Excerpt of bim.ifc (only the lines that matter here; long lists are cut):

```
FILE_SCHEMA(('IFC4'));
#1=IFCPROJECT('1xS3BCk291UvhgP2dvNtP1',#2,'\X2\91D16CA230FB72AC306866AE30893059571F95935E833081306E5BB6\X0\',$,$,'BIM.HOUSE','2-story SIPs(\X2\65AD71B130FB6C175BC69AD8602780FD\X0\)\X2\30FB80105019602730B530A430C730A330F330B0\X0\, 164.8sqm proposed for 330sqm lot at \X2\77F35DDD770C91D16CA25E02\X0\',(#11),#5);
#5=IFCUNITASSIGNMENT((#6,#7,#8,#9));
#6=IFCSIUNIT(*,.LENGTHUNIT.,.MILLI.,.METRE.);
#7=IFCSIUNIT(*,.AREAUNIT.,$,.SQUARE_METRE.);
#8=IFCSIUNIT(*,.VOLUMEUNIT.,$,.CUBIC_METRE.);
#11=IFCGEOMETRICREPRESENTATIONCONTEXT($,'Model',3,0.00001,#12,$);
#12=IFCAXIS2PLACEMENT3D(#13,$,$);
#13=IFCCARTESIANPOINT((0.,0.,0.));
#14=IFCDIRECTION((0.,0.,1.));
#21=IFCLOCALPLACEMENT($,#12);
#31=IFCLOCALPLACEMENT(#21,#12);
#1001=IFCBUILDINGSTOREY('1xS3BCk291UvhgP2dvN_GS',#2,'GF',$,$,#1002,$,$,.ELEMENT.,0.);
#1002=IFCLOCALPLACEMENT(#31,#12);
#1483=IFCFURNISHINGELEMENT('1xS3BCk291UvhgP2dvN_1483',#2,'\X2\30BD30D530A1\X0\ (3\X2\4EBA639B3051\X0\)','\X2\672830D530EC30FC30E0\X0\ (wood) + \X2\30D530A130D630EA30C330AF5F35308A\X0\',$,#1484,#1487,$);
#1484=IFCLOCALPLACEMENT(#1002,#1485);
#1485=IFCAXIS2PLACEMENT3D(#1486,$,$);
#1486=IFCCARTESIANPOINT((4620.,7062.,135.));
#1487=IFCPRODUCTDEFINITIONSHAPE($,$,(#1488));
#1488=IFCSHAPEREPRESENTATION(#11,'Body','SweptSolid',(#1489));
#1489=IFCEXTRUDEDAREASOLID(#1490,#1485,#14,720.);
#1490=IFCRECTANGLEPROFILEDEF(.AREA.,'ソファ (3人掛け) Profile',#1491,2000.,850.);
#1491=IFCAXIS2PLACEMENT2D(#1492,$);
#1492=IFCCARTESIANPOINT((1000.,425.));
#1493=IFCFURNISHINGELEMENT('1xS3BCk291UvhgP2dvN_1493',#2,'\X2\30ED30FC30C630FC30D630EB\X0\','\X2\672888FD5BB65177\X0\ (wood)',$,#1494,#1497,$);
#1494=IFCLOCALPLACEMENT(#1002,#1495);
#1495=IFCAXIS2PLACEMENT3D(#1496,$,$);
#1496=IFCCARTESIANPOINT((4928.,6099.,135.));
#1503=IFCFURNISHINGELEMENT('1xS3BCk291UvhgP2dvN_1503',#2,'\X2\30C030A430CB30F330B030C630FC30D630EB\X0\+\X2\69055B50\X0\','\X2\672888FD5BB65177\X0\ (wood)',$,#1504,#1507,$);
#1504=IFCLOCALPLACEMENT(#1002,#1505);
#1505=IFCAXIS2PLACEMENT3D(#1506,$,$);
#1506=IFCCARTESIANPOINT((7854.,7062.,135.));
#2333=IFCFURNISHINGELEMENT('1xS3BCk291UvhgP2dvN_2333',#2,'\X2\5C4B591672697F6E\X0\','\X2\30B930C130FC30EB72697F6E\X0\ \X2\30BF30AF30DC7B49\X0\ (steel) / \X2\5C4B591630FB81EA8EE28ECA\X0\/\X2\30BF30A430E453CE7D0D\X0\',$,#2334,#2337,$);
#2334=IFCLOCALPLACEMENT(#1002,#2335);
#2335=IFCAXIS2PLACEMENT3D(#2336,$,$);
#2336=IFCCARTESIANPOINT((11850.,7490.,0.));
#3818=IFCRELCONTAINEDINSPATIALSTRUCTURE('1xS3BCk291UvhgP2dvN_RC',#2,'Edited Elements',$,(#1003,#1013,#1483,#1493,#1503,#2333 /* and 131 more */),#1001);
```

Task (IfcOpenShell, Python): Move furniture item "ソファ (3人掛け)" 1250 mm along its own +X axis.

```python
import ifcopenshell
import ifcopenshell.api.geometry
import ifcopenshell.util.placement
import ifcopenshell.util.unit

model = ifcopenshell.open("bim.ifc")
unit_scale = ifcopenshell.util.unit.calculate_unit_scale(model)

item = model.by_id(1483)
matrix = ifcopenshell.util.placement.get_local_placement(item.ObjectPlacement)
matrix[:3, 3] += matrix[:3, 0] * 1.25 / unit_scale
ifcopenshell.api.geometry.edit_object_placement(model, product=item, matrix=matrix, is_si=False)

print(ifcopenshell.util.placement.get_local_placement(item.ObjectPlacement).round(3) + 0.0)

model.write("bim_v2.ifc")
```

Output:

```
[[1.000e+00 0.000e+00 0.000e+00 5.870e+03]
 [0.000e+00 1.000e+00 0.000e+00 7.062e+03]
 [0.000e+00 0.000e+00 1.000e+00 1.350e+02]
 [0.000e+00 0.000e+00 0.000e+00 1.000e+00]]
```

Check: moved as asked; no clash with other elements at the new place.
